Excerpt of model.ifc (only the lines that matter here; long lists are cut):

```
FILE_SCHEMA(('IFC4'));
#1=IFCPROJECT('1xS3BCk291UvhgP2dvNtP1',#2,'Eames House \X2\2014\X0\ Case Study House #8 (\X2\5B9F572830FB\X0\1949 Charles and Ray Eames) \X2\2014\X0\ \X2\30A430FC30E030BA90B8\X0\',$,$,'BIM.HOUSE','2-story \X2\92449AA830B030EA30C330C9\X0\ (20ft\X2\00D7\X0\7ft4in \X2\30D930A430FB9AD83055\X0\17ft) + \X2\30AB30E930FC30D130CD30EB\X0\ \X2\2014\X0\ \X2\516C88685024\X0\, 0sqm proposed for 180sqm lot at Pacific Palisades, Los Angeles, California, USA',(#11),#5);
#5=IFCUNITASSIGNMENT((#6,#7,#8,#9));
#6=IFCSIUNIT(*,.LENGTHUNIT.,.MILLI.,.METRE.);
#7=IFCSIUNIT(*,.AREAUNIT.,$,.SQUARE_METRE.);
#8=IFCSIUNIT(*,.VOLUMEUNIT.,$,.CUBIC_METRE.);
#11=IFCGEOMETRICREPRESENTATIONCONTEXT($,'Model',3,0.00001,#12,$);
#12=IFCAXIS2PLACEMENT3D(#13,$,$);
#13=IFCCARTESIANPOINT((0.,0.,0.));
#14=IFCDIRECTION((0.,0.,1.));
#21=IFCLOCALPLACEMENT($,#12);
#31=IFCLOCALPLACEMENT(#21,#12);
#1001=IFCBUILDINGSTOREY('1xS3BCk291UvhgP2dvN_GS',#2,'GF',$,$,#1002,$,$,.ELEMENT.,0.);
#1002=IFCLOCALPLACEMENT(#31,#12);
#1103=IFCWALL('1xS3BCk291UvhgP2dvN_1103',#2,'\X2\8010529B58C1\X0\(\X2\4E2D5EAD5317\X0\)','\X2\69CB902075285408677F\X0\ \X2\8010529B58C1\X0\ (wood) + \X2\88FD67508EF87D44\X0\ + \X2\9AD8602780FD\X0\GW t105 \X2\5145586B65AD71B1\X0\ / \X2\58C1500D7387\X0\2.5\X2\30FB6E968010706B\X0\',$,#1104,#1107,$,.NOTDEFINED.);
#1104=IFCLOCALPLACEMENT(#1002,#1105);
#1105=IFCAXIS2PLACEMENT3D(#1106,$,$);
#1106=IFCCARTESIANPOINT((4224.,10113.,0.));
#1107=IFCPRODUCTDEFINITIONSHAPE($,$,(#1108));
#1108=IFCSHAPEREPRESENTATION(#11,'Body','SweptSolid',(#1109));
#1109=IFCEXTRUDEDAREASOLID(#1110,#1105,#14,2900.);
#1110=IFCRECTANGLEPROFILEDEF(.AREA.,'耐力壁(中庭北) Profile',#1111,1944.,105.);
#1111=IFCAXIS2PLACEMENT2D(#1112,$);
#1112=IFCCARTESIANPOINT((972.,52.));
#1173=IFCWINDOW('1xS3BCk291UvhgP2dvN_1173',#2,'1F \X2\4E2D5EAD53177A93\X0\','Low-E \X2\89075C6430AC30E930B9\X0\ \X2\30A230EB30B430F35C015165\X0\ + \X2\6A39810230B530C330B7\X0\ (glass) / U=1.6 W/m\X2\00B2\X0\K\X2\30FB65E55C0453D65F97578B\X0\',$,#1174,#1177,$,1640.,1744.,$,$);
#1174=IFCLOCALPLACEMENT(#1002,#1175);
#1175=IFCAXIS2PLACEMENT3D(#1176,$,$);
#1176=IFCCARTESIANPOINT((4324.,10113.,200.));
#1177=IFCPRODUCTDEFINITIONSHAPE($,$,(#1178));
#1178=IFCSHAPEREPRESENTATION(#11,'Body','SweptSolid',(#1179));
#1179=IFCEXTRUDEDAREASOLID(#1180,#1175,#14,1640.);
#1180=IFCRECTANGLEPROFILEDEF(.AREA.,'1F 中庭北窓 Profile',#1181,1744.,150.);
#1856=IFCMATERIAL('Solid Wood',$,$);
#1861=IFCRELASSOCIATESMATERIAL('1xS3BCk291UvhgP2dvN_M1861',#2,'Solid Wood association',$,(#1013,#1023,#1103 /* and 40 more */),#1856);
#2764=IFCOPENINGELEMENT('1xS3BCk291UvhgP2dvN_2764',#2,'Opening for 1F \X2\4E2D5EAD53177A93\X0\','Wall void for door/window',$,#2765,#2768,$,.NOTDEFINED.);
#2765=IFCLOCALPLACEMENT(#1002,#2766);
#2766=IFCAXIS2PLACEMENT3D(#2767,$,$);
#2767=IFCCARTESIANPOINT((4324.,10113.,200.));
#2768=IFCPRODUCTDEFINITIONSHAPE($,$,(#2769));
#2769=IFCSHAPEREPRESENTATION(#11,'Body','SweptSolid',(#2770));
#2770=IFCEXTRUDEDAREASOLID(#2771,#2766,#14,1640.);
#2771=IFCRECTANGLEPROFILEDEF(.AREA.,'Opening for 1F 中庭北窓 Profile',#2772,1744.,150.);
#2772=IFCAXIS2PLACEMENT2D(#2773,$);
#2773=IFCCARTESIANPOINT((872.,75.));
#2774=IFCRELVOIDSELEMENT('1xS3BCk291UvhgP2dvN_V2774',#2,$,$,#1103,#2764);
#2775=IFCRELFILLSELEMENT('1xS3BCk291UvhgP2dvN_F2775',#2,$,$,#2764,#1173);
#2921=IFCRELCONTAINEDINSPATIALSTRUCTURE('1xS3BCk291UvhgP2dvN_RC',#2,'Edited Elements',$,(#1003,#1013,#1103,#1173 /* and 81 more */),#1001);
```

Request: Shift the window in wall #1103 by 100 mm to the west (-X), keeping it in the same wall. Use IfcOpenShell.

```python
import ifcopenshell
import ifcopenshell.api.geometry
import ifcopenshell.util.placement
import ifcopenshell.util.unit

model = ifcopenshell.open("model.ifc")
unit_scale = ifcopenshell.util.unit.calculate_unit_scale(model)

window = model.by_guid("1xS3BCk291UvhgP2dvN_1173")
opening = window.FillsVoids[0].RelatingOpeningElement
wall = opening.VoidsElements[0].RelatingBuildingElement

wall_matrix = ifcopenshell.util.placement.get_local_placement(wall.ObjectPlacement)
shift = wall_matrix[:3, 0] * -0.1 / unit_scale
before = ifcopenshell.util.placement.get_local_placement(window.ObjectPlacement)[:3, 3].copy()

# The window is not placed relative to its opening, so move both.
for product in (opening, window):
    matrix = ifcopenshell.util.placement.get_local_placement(product.ObjectPlacement)
    matrix[:3, 3] += shift
    ifcopenshell.api.geometry.edit_object_placement(model, product=product, matrix=matrix, is_si=False)

after = ifcopenshell.util.placement.get_local_placement(window.ObjectPlacement)[:3, 3]
print("window moved by", (after - before).round(3) + 0.0)

model.write("model_updated.ifc")
```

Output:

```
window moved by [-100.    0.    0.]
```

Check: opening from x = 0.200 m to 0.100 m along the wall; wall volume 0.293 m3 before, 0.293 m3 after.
